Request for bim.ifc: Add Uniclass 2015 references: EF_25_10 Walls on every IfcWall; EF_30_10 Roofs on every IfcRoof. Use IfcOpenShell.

First a look at what the model holds.

```python
import ifcopenshell

model = ifcopenshell.open("bim.ifc")
print(model.schema)
print("classifications:", [c.Name for c in model.by_type("IfcClassification")])
for ifc_class in ("IfcDoor", "IfcRoof", "IfcStair", "IfcWall", "IfcWindow"):
    print(ifc_class, len(model.by_type(ifc_class)))
```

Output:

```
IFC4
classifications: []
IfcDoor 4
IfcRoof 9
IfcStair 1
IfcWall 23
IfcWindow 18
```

```python
import ifcopenshell
import ifcopenshell.api.classification

model = ifcopenshell.open("bim.ifc")

system = ifcopenshell.api.classification.add_classification(model, classification="Uniclass 2015")

codes = {
    "IfcWall": ("EF_25_10", "Walls"),
    "IfcRoof": ("EF_30_10", "Roofs"),
}
for ifc_class, (code, name) in codes.items():
    products = model.by_type(ifc_class)
    ifcopenshell.api.classification.add_reference(
        model, products=products, classification=system, identification=code, name=name
    )
    print(code, len(products))

model.write("bim-out.ifc")
```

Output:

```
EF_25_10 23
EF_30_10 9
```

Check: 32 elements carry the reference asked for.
